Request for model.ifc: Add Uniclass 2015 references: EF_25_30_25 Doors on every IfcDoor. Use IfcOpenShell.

First a look at what the model holds.

```python
import ifcopenshell

model = ifcopenshell.open("model.ifc")
print(model.schema)
print("classifications:", [c.Name for c in model.by_type("IfcClassification")])
for ifc_class in ("IfcDoor", "IfcRoof", "IfcStair", "IfcWall", "IfcWindow"):
    print(ifc_class, len(model.by_type(ifc_class)))
```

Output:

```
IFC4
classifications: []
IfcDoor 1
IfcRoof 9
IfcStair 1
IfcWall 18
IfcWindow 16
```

```python
import ifcopenshell
import ifcopenshell.api.classification

model = ifcopenshell.open("model.ifc")

system = ifcopenshell.api.classification.add_classification(model, classification="Uniclass 2015")

codes = {
    "IfcDoor": ("EF_25_30_25", "Doors"),
}
for ifc_class, (code, name) in codes.items():
    products = model.by_type(ifc_class)
    ifcopenshell.api.classification.add_reference(
        model, products=products, classification=system, identification=code, name=name
    )
    print(code, len(products))

model.write("model-out.ifc")
```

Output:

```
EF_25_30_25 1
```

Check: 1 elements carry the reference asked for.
